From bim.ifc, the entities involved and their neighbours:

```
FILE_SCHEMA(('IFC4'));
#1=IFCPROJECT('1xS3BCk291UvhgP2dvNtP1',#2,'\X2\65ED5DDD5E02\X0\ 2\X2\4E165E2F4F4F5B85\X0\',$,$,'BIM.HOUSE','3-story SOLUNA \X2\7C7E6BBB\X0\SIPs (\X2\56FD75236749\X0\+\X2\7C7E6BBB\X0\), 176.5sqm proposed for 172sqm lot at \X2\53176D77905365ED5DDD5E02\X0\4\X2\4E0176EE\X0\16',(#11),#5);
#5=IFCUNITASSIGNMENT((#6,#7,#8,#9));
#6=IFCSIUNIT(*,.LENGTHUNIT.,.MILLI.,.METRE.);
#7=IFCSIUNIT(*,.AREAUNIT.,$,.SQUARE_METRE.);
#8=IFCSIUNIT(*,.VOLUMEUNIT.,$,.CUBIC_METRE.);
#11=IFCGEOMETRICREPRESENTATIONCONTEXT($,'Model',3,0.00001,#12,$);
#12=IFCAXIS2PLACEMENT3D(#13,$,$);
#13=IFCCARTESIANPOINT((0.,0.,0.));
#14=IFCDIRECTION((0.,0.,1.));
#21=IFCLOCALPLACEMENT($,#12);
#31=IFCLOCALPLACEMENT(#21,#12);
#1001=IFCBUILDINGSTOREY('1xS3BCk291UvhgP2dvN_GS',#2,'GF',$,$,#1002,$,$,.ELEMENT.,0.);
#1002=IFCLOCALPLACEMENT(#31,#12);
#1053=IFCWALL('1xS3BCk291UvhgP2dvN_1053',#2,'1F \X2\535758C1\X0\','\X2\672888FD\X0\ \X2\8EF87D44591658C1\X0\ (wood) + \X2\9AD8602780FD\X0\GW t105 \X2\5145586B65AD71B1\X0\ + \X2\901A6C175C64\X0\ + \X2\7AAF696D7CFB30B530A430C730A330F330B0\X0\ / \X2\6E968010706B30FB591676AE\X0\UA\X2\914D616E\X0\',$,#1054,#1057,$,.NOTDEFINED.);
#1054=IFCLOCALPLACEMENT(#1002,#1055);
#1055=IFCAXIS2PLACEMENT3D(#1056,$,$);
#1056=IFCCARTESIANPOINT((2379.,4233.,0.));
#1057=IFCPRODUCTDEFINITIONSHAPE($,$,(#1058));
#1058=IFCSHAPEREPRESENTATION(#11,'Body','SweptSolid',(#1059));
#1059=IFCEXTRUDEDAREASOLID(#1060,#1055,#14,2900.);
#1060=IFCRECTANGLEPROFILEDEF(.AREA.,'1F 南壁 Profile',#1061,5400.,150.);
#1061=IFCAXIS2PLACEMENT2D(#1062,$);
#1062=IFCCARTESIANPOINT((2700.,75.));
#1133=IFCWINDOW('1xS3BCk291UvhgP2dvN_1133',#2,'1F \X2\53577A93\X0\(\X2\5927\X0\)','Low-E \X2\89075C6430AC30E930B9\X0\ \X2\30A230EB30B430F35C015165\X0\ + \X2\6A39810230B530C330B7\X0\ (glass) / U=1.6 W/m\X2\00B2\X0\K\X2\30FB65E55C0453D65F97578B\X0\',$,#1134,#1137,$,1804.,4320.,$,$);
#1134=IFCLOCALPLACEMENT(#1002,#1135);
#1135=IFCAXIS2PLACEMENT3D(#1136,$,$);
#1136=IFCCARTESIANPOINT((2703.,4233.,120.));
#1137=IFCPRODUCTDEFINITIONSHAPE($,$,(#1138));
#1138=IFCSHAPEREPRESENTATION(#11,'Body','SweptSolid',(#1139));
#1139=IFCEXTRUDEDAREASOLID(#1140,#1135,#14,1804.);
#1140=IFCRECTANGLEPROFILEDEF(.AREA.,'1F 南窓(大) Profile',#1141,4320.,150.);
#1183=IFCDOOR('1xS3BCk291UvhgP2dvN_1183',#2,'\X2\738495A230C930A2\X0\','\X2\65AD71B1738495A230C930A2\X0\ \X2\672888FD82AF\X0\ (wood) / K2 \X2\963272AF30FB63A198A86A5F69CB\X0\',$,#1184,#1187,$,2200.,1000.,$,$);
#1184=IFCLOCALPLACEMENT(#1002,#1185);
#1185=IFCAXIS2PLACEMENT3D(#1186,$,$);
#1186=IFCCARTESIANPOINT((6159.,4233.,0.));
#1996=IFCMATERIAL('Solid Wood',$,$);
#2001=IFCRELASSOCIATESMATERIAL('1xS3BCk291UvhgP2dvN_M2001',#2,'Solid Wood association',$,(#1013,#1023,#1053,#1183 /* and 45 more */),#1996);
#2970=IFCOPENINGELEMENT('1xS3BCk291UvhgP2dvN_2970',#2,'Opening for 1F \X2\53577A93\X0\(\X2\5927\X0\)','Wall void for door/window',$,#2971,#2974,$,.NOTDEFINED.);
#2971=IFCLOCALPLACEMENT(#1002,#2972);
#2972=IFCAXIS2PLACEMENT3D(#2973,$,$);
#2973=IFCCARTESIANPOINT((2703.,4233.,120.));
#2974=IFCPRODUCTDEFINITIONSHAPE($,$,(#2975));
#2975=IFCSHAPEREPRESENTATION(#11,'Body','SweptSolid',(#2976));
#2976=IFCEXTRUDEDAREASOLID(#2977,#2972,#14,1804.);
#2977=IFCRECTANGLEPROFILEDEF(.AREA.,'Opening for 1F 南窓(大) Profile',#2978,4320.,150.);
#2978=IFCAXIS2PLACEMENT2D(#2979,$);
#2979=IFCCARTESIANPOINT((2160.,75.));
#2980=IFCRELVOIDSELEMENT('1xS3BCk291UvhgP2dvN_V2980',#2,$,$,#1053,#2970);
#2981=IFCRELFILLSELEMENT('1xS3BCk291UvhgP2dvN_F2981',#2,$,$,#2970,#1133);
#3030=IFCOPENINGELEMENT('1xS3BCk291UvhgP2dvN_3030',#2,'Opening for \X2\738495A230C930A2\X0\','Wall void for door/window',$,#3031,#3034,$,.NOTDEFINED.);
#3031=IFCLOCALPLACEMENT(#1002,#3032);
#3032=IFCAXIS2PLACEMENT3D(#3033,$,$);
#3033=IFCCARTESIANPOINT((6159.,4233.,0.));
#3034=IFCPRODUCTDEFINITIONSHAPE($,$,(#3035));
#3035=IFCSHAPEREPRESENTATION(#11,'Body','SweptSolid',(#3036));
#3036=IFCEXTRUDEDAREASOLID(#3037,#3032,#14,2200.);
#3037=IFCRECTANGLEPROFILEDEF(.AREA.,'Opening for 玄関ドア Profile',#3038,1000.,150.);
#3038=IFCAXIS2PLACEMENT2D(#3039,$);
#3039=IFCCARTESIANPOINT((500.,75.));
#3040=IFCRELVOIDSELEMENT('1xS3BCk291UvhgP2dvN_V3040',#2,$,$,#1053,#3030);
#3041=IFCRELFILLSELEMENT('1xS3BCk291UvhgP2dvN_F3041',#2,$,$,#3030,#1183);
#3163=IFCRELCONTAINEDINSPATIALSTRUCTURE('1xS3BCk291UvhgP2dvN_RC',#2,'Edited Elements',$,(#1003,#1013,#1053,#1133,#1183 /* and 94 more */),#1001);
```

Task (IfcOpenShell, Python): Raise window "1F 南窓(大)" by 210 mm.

```python
import numpy as np
import ifcopenshell
import ifcopenshell.api.geometry
import ifcopenshell.util.placement
import ifcopenshell.util.unit

model = ifcopenshell.open("bim.ifc")
unit_scale = ifcopenshell.util.unit.calculate_unit_scale(model)

window = model.by_guid("1xS3BCk291UvhgP2dvN_1133")
opening = window.FillsVoids[0].RelatingOpeningElement
dz = 0.21 / unit_scale

shift = np.array([0.0, 0.0, dz])
# The window is not placed relative to its opening, so move both.
for product in (opening, window):
    matrix = ifcopenshell.util.placement.get_local_placement(product.ObjectPlacement)
    matrix[:3, 3] += shift
    ifcopenshell.api.geometry.edit_object_placement(model, product=product, matrix=matrix, is_si=False)

print(f"moved by {dz * unit_scale:+.3f} m")

model.write("bim_edited.ifc")
```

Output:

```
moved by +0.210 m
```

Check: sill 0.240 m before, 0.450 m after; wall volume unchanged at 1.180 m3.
